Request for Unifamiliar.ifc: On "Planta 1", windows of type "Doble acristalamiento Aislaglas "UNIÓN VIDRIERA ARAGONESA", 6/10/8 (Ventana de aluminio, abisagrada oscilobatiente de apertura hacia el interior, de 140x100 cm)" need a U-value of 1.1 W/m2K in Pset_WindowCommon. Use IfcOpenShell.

First a look at what the model holds.

```python
import ifcopenshell
import ifcopenshell.util.element

model = ifcopenshell.open("Unifamiliar.ifc")
print(model.schema)
storey = next(s for s in model.by_type("IfcBuildingStorey") if s.Name == "Planta 1")
windows = [e for e in ifcopenshell.util.element.get_decomposition(storey) if e.is_a("IfcWindow")]
seen = {}
for e in windows:
    element_type = ifcopenshell.util.element.get_type(e)
    key = (element_type.Name if element_type != e and element_type else None, ifcopenshell.util.element.get_pset(e, "Pset_WindowCommon", "ThermalTransmittance"))
    seen[key] = seen.get(key, 0) + 1
for (name, value), count in sorted(seen.items(), key=str):
    print(count, "x", name, "|", value)
```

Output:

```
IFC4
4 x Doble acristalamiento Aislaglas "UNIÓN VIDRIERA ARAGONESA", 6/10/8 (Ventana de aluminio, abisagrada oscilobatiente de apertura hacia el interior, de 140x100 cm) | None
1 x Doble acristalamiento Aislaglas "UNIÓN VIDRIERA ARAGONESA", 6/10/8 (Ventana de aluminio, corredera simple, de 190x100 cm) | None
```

```python
import ifcopenshell
import ifcopenshell.api.pset
import ifcopenshell.util.element

model = ifcopenshell.open("Unifamiliar.ifc")

storey = next(s for s in model.by_type("IfcBuildingStorey") if s.Name == "Planta 1")
windows = [e for e in ifcopenshell.util.element.get_decomposition(storey) if e.is_a("IfcWindow")]

count = 0
for e in windows:
    element_type = ifcopenshell.util.element.get_type(e)
    if element_type in (None, e) or element_type.Name != 'Doble acristalamiento Aislaglas "UNIÓN VIDRIERA ARAGONESA", 6/10/8 (Ventana de aluminio, abisagrada oscilobatiente de apertura hacia el interior, de 140x100 cm)':
        continue
    # add_pset returns the element's existing set when there is one.
    pset = ifcopenshell.api.pset.add_pset(model, product=e, name="Pset_WindowCommon")
    ifcopenshell.api.pset.edit_pset(model, pset=pset, properties={"ThermalTransmittance": 1.1})
    count += 1

print(count, "windows updated")

model.write("Unifamiliar-out.ifc")
```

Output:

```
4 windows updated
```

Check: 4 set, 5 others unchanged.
